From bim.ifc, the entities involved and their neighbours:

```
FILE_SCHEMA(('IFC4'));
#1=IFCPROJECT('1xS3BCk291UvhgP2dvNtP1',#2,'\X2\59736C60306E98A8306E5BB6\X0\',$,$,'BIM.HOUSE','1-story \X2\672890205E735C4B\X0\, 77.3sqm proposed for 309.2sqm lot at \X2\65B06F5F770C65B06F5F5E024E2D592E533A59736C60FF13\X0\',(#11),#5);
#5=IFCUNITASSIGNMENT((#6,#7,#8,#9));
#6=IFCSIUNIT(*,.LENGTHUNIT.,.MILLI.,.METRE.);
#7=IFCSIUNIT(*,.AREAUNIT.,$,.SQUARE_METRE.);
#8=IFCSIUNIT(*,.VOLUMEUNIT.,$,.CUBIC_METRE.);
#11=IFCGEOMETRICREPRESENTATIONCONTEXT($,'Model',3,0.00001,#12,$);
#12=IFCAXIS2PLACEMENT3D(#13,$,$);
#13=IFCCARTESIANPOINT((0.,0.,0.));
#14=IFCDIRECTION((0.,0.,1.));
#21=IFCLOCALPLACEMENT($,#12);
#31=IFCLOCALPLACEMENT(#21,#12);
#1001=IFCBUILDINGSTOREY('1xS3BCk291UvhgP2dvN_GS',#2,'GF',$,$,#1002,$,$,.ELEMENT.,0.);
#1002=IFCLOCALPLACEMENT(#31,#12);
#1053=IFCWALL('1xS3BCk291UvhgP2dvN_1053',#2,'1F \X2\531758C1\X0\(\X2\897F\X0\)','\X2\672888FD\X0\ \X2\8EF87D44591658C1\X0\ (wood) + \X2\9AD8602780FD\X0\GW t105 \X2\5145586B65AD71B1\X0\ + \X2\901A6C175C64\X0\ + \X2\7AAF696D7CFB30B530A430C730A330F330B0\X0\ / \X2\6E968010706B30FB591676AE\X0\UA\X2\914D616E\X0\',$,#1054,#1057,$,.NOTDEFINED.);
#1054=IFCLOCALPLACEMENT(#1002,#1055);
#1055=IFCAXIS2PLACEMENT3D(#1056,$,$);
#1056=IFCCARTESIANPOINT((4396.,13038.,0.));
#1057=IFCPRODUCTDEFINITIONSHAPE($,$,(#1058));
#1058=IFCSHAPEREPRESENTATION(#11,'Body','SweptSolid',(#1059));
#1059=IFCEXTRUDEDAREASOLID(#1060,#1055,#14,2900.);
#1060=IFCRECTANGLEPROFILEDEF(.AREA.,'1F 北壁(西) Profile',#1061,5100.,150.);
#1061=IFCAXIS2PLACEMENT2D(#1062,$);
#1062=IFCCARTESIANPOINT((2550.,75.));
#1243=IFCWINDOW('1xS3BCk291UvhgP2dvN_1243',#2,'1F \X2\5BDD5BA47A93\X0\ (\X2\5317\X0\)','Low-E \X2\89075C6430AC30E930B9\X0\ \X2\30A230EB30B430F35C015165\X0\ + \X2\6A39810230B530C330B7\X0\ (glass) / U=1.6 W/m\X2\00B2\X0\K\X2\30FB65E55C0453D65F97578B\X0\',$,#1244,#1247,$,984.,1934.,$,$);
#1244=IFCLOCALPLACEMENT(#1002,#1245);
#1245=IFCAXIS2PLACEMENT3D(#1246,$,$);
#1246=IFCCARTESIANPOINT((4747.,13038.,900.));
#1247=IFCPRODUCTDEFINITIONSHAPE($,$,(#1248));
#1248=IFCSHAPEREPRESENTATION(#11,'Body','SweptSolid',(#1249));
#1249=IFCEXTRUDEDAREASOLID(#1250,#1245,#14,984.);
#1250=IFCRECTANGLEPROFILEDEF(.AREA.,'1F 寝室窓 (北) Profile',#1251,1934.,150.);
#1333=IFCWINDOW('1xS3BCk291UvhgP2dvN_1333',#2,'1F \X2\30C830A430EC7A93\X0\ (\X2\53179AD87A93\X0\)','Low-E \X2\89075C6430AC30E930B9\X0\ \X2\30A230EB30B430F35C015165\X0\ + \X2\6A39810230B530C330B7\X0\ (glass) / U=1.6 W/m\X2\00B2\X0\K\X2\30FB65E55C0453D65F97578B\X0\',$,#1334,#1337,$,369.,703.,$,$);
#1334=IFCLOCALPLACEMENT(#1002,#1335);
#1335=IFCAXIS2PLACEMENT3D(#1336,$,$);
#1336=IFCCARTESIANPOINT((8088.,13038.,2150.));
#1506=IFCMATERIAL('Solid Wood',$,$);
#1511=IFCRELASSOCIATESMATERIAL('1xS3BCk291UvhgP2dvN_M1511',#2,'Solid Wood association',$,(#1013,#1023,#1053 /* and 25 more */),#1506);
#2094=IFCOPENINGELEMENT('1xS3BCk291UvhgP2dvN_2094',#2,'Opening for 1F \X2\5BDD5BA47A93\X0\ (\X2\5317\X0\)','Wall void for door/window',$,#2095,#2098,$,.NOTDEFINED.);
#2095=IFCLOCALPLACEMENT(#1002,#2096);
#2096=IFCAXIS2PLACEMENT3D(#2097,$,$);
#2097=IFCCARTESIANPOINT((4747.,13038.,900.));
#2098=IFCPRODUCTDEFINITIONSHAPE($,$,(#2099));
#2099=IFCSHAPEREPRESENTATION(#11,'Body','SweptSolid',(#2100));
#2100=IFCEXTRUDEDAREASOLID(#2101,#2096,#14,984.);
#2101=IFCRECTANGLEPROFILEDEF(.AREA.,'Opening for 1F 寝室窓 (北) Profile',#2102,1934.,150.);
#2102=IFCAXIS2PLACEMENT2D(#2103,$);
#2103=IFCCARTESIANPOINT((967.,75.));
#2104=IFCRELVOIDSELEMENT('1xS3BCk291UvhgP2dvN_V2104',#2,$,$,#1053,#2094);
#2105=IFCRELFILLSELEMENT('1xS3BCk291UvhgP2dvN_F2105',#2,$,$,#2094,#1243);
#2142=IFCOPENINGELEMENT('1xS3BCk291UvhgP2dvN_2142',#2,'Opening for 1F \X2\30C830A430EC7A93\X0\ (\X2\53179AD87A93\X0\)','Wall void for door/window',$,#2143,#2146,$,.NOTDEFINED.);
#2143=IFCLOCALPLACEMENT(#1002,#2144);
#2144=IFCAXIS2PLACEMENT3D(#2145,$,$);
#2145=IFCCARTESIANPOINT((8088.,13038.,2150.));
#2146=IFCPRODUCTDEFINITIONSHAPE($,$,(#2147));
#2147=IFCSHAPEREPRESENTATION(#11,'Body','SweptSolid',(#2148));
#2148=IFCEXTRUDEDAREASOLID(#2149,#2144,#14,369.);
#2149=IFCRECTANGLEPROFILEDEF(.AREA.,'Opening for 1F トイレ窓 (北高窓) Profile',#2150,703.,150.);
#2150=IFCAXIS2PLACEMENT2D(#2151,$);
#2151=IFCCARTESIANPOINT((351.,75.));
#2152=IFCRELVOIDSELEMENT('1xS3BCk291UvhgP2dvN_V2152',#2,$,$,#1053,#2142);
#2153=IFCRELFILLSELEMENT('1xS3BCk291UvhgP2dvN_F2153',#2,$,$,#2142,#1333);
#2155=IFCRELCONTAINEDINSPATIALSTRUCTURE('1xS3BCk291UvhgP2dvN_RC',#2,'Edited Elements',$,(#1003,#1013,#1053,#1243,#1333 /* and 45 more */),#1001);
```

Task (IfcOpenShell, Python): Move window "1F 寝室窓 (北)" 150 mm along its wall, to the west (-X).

```python
import ifcopenshell
import ifcopenshell.api.geometry
import ifcopenshell.util.placement
import ifcopenshell.util.unit

model = ifcopenshell.open("bim.ifc")
unit_scale = ifcopenshell.util.unit.calculate_unit_scale(model)

window = model.by_id(1243)
opening = window.FillsVoids[0].RelatingOpeningElement
wall = opening.VoidsElements[0].RelatingBuildingElement

wall_matrix = ifcopenshell.util.placement.get_local_placement(wall.ObjectPlacement)
shift = wall_matrix[:3, 0] * -0.15 / unit_scale
before = ifcopenshell.util.placement.get_local_placement(window.ObjectPlacement)[:3, 3].copy()

# The window is not placed relative to its opening, so move both.
for product in (opening, window):
    matrix = ifcopenshell.util.placement.get_local_placement(product.ObjectPlacement)
    matrix[:3, 3] += shift
    ifcopenshell.api.geometry.edit_object_placement(model, product=product, matrix=matrix, is_si=False)

after = ifcopenshell.util.placement.get_local_placement(window.ObjectPlacement)[:3, 3]
print("window moved by", (after - before).round(3) + 0.0)

model.write("bim-out.ifc")
```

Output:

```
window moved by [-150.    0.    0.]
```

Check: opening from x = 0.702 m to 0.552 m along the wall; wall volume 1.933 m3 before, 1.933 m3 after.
